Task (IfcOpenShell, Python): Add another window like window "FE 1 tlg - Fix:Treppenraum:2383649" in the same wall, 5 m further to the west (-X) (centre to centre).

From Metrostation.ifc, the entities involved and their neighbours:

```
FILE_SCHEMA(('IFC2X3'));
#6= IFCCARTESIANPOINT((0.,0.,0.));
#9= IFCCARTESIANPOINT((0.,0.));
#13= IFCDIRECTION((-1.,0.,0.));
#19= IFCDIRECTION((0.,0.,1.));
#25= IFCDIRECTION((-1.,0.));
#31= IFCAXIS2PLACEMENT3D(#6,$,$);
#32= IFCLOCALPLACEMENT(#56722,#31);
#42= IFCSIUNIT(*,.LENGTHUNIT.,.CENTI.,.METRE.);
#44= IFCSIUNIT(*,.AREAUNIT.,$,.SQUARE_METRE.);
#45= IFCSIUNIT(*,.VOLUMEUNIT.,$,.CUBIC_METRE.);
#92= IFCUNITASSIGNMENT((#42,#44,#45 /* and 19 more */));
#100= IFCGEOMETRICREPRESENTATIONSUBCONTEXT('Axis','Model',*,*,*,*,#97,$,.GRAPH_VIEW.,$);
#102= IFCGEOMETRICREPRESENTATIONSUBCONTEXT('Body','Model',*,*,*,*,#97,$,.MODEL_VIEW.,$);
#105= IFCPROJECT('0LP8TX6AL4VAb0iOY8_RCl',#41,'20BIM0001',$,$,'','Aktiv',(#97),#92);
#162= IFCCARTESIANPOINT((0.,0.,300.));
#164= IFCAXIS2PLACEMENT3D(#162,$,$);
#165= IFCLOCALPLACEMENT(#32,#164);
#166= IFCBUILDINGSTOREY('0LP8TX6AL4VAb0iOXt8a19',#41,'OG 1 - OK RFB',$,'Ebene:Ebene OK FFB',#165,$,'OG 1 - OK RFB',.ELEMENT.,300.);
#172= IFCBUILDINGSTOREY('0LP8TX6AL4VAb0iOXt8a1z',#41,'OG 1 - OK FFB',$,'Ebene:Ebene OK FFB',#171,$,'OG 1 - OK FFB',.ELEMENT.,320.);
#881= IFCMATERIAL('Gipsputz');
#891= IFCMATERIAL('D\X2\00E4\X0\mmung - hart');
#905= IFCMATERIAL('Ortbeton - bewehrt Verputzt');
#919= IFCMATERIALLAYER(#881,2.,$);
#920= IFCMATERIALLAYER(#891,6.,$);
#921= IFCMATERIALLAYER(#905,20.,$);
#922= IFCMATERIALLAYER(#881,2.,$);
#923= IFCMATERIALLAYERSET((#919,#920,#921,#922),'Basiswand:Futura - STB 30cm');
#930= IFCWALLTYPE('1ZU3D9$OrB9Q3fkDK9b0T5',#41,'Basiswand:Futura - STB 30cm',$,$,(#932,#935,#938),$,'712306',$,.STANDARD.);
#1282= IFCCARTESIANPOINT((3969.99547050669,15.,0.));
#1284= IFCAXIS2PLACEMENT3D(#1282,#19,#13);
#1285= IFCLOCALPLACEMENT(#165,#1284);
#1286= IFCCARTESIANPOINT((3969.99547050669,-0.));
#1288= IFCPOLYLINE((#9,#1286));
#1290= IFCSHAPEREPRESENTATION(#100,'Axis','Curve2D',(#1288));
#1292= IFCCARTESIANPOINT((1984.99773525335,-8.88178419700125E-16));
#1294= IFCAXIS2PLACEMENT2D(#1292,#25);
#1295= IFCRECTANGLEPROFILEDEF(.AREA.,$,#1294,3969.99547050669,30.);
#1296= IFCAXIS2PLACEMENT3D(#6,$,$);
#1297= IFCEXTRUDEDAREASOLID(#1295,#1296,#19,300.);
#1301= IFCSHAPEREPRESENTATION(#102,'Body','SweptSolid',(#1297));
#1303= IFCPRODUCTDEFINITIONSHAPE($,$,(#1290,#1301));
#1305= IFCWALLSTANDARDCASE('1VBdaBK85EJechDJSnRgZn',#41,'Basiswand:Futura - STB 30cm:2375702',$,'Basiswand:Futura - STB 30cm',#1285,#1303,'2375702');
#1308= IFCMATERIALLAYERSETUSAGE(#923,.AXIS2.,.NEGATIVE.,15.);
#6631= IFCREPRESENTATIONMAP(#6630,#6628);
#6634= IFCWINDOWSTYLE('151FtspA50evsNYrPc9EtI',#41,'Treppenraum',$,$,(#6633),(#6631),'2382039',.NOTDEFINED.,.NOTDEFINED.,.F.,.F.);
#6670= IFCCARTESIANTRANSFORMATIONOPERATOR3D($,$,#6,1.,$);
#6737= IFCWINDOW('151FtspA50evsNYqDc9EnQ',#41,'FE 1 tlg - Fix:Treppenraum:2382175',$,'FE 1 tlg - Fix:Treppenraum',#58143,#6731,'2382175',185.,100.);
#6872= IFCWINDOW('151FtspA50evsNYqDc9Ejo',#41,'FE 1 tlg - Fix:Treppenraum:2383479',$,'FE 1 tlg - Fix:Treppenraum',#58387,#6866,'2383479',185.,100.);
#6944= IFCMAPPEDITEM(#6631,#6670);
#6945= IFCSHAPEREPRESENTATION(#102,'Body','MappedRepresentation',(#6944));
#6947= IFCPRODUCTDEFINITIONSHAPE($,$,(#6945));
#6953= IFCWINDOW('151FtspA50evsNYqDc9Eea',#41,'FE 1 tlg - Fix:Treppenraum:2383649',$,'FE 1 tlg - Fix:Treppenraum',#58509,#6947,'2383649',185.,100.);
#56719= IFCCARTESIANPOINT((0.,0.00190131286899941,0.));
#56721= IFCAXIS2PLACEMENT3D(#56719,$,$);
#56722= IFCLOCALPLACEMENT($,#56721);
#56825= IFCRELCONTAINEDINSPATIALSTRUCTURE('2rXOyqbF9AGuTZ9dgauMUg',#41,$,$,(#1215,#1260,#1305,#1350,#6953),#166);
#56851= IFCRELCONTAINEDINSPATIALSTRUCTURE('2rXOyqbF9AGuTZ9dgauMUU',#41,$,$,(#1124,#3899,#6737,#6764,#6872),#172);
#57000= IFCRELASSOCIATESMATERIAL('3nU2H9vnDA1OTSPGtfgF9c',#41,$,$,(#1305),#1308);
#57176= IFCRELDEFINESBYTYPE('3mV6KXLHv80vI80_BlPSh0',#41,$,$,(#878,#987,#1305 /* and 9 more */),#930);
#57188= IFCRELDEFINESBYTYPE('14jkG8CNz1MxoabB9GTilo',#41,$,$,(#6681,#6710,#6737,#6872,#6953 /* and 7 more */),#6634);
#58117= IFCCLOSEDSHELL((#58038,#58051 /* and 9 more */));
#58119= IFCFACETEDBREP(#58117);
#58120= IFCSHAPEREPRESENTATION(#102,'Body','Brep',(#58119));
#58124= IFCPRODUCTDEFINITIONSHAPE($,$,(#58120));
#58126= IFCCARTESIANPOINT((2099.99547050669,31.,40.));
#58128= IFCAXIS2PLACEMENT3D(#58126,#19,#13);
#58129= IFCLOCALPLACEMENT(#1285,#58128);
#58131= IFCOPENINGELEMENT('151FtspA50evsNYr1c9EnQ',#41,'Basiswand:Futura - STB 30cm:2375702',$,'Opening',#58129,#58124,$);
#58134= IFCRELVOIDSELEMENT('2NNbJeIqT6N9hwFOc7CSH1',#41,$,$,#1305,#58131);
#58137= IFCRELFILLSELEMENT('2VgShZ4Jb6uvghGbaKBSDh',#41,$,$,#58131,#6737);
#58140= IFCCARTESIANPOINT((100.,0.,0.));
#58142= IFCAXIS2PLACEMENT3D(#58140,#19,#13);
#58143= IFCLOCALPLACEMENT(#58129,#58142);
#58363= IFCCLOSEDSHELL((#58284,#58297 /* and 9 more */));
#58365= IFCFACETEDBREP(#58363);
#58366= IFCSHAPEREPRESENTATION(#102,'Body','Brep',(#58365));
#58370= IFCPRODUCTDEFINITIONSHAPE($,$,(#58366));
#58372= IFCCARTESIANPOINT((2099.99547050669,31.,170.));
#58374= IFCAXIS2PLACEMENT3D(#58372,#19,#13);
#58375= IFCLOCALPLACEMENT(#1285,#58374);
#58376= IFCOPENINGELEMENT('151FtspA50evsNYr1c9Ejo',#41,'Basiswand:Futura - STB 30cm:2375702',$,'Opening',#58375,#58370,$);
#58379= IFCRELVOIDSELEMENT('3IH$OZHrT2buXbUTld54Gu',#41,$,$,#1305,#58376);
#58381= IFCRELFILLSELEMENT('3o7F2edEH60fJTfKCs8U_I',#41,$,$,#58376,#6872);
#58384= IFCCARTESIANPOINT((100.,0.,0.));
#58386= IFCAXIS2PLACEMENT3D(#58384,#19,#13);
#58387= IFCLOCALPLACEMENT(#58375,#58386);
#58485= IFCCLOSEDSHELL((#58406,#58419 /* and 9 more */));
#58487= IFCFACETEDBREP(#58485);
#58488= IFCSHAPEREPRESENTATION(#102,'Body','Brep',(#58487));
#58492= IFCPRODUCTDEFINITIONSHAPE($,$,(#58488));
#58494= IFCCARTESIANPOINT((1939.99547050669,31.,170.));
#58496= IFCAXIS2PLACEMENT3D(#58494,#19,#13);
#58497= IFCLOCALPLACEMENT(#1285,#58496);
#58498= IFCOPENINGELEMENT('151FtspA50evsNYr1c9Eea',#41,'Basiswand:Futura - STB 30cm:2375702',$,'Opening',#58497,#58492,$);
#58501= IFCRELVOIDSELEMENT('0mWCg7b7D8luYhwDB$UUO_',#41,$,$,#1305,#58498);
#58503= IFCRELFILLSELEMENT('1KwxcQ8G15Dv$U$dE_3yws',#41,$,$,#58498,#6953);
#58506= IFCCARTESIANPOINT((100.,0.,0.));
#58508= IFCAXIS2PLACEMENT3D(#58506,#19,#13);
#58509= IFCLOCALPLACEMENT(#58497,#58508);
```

```python
import ifcopenshell
import ifcopenshell.api.feature
import ifcopenshell.api.geometry
import ifcopenshell.api.root
import ifcopenshell.geom
import ifcopenshell.util.element
import ifcopenshell.util.placement
import ifcopenshell.util.shape
import ifcopenshell.util.unit

model = ifcopenshell.open("Metrostation.ifc")
unit_scale = ifcopenshell.util.unit.calculate_unit_scale(model)
settings = ifcopenshell.geom.settings()


def volume(element):
    """Net volume in cubic metres, openings subtracted."""
    shape = ifcopenshell.geom.create_shape(settings, element)
    return ifcopenshell.util.shape.get_volume(shape.geometry)


def reuse_history(source, copy):
    """copy_class also copies each property set's owner history, people and application; keep the originals."""
    for rel in copy.IsDefinedBy:
        if rel.is_a("IfcRelDefinesByProperties") and (history := rel.RelatingPropertyDefinition.OwnerHistory):
            rel.RelatingPropertyDefinition.OwnerHistory = source.OwnerHistory
            ifcopenshell.util.element.remove_deep2(model, history)


window = model.by_guid("151FtspA50evsNYqDc9Eea")
opening = window.FillsVoids[0].RelatingOpeningElement
wall = opening.VoidsElements[0].RelatingBuildingElement
before = volume(wall)
shift = ifcopenshell.util.placement.get_local_placement(wall.ObjectPlacement)[:3, 0] * 5 / unit_scale

# copy_class copies the void relationship, type, container and properties, but no geometry.
new_opening = ifcopenshell.api.root.copy_class(model, product=opening)
new_opening.Representation = ifcopenshell.util.element.copy_deep(
    model, opening.Representation, exclude=["IfcGeometricRepresentationContext", "IfcRepresentationMap"]
)
new_opening.Name = "Basiswand:Futura - STB 30cm"
new_window = ifcopenshell.api.root.copy_class(model, product=window)
new_window.Representation = ifcopenshell.util.element.copy_deep(
    model, window.Representation, exclude=["IfcGeometricRepresentationContext", "IfcRepresentationMap"]
)
new_window.Name = "FE 1 tlg - Fix:Treppenraum"
new_window.Tag = None
reuse_history(window, new_window)
fills = ifcopenshell.api.feature.add_filling(model, opening=new_opening, element=new_window)
fills.OwnerHistory = new_window.OwnerHistory  # required in IFC2X3

for old, new in ((opening, new_opening), (window, new_window)):
    matrix = ifcopenshell.util.placement.get_local_placement(old.ObjectPlacement)
    matrix[:3, 3] += shift
    ifcopenshell.api.geometry.edit_object_placement(model, product=new, matrix=matrix, is_si=False)

after = volume(wall)

print(f"wall volume {before:.3f} -> {after:.3f} m3")

model.write("Metrostation_edited.ifc")
```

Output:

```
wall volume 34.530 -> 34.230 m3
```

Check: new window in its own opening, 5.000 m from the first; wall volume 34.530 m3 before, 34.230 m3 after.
